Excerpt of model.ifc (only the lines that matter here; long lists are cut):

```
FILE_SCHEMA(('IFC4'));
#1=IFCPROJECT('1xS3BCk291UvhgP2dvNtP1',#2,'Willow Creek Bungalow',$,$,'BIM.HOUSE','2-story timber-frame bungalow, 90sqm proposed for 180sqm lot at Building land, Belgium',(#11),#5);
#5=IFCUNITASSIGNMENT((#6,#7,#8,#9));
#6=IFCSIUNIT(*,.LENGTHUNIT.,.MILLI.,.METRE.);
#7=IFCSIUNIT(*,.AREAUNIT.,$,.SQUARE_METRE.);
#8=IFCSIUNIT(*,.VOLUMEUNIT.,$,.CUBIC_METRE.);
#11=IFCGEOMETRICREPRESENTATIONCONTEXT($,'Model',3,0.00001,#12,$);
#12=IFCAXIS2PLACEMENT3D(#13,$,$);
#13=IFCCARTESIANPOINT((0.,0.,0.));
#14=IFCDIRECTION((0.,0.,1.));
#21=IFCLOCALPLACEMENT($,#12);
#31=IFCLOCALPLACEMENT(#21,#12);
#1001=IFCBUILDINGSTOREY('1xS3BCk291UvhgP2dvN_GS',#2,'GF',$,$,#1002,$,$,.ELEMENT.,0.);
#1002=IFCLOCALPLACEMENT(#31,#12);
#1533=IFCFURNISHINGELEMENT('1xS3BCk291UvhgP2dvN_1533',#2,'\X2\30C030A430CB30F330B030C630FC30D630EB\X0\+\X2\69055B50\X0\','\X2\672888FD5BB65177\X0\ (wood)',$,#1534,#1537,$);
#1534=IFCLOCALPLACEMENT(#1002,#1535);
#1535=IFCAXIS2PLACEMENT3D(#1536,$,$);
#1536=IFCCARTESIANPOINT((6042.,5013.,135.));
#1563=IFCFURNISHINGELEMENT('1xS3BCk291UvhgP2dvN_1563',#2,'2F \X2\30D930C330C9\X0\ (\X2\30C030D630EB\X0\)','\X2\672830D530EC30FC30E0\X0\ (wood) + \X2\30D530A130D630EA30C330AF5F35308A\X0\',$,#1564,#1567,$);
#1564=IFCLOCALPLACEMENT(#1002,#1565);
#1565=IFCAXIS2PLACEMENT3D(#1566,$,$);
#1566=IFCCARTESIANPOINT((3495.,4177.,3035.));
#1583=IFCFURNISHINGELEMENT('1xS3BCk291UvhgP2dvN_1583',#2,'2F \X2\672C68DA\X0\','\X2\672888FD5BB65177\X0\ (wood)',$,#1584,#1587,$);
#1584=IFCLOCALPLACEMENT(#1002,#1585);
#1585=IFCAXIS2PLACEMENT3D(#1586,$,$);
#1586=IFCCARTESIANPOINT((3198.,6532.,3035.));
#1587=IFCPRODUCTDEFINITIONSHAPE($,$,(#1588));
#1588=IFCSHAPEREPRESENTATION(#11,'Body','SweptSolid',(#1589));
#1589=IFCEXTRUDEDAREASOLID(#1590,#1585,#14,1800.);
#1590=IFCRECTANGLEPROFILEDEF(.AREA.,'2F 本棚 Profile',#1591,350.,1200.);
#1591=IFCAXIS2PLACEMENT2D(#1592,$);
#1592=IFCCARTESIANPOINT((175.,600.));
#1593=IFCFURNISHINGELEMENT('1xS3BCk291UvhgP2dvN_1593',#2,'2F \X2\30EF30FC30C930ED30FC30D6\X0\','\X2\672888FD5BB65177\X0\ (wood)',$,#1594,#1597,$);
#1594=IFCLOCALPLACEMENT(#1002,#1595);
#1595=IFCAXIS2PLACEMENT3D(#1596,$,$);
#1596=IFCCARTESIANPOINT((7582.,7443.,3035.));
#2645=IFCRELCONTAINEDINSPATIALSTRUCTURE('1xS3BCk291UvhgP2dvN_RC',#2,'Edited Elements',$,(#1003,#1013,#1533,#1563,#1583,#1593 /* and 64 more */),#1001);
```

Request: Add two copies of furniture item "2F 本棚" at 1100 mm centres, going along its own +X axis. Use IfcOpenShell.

```python
import ifcopenshell
import ifcopenshell.api.geometry
import ifcopenshell.api.root
import ifcopenshell.util.element
import ifcopenshell.util.placement
import ifcopenshell.util.unit

model = ifcopenshell.open("model.ifc")
unit_scale = ifcopenshell.util.unit.calculate_unit_scale(model)


def reuse_history(source, copy):
    """copy_class also copies each property set's owner history, people and application; keep the originals."""
    for rel in copy.IsDefinedBy:
        if rel.is_a("IfcRelDefinesByProperties") and (history := rel.RelatingPropertyDefinition.OwnerHistory):
            rel.RelatingPropertyDefinition.OwnerHistory = source.OwnerHistory
            ifcopenshell.util.element.remove_deep2(model, history)


source = model.by_guid("1xS3BCk291UvhgP2dvN_1583")
base = ifcopenshell.util.placement.get_local_placement(source.ObjectPlacement)
step = base[:3, 0] * 1.1 / unit_scale

for i in range(1, 3):
    copy = ifcopenshell.api.root.copy_class(model, product=source)
    copy.Representation = ifcopenshell.util.element.copy_deep(
        model, source.Representation, exclude=["IfcGeometricRepresentationContext", "IfcRepresentationMap"]
    )
    reuse_history(source, copy)
    matrix = base.copy()
    matrix[:3, 3] += i * step
    print("added at", matrix[:3, 3].round(3) + 0.0)
    ifcopenshell.api.geometry.edit_object_placement(model, product=copy, matrix=matrix, is_si=False)

model.write("model_rev.ifc")
```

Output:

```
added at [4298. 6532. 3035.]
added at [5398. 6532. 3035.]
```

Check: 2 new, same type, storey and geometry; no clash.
